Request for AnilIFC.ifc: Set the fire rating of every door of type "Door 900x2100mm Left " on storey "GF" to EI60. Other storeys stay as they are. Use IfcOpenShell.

First a look at what the model holds.

```python
import ifcopenshell
import ifcopenshell.util.element

model = ifcopenshell.open("AnilIFC.ifc")
print(model.schema)
storey = next(s for s in model.by_type("IfcBuildingStorey") if s.Name == "GF")
doors = [e for e in ifcopenshell.util.element.get_decomposition(storey) if e.is_a("IfcDoor")]
seen = {}
for e in doors:
    element_type = ifcopenshell.util.element.get_type(e)
    key = (element_type.Name if element_type != e and element_type else None, ifcopenshell.util.element.get_pset(e, "Pset_DoorCommon", "FireRating"))
    seen[key] = seen.get(key, 0) + 1
for (name, value), count in sorted(seen.items(), key=str):
    print(count, "x", name, "|", value)
```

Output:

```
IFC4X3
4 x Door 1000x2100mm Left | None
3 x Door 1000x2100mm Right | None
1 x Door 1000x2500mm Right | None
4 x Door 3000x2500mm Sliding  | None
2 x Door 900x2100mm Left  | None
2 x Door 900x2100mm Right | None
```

```python
import ifcopenshell
import ifcopenshell.api.pset
import ifcopenshell.util.element

model = ifcopenshell.open("AnilIFC.ifc")

storey = next(s for s in model.by_type("IfcBuildingStorey") if s.Name == "GF")
doors = [e for e in ifcopenshell.util.element.get_decomposition(storey) if e.is_a("IfcDoor")]

count = 0
for e in doors:
    element_type = ifcopenshell.util.element.get_type(e)
    if element_type in (None, e) or element_type.Name != "Door 900x2100mm Left ":
        continue
    # add_pset returns the element's existing set when there is one.
    pset = ifcopenshell.api.pset.add_pset(model, product=e, name="Pset_DoorCommon")
    ifcopenshell.api.pset.edit_pset(model, pset=pset, properties={"FireRating": "EI60"})
    count += 1

print(count, "doors updated")

model.write("AnilIFC-out.ifc")
```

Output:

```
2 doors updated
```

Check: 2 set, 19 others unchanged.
